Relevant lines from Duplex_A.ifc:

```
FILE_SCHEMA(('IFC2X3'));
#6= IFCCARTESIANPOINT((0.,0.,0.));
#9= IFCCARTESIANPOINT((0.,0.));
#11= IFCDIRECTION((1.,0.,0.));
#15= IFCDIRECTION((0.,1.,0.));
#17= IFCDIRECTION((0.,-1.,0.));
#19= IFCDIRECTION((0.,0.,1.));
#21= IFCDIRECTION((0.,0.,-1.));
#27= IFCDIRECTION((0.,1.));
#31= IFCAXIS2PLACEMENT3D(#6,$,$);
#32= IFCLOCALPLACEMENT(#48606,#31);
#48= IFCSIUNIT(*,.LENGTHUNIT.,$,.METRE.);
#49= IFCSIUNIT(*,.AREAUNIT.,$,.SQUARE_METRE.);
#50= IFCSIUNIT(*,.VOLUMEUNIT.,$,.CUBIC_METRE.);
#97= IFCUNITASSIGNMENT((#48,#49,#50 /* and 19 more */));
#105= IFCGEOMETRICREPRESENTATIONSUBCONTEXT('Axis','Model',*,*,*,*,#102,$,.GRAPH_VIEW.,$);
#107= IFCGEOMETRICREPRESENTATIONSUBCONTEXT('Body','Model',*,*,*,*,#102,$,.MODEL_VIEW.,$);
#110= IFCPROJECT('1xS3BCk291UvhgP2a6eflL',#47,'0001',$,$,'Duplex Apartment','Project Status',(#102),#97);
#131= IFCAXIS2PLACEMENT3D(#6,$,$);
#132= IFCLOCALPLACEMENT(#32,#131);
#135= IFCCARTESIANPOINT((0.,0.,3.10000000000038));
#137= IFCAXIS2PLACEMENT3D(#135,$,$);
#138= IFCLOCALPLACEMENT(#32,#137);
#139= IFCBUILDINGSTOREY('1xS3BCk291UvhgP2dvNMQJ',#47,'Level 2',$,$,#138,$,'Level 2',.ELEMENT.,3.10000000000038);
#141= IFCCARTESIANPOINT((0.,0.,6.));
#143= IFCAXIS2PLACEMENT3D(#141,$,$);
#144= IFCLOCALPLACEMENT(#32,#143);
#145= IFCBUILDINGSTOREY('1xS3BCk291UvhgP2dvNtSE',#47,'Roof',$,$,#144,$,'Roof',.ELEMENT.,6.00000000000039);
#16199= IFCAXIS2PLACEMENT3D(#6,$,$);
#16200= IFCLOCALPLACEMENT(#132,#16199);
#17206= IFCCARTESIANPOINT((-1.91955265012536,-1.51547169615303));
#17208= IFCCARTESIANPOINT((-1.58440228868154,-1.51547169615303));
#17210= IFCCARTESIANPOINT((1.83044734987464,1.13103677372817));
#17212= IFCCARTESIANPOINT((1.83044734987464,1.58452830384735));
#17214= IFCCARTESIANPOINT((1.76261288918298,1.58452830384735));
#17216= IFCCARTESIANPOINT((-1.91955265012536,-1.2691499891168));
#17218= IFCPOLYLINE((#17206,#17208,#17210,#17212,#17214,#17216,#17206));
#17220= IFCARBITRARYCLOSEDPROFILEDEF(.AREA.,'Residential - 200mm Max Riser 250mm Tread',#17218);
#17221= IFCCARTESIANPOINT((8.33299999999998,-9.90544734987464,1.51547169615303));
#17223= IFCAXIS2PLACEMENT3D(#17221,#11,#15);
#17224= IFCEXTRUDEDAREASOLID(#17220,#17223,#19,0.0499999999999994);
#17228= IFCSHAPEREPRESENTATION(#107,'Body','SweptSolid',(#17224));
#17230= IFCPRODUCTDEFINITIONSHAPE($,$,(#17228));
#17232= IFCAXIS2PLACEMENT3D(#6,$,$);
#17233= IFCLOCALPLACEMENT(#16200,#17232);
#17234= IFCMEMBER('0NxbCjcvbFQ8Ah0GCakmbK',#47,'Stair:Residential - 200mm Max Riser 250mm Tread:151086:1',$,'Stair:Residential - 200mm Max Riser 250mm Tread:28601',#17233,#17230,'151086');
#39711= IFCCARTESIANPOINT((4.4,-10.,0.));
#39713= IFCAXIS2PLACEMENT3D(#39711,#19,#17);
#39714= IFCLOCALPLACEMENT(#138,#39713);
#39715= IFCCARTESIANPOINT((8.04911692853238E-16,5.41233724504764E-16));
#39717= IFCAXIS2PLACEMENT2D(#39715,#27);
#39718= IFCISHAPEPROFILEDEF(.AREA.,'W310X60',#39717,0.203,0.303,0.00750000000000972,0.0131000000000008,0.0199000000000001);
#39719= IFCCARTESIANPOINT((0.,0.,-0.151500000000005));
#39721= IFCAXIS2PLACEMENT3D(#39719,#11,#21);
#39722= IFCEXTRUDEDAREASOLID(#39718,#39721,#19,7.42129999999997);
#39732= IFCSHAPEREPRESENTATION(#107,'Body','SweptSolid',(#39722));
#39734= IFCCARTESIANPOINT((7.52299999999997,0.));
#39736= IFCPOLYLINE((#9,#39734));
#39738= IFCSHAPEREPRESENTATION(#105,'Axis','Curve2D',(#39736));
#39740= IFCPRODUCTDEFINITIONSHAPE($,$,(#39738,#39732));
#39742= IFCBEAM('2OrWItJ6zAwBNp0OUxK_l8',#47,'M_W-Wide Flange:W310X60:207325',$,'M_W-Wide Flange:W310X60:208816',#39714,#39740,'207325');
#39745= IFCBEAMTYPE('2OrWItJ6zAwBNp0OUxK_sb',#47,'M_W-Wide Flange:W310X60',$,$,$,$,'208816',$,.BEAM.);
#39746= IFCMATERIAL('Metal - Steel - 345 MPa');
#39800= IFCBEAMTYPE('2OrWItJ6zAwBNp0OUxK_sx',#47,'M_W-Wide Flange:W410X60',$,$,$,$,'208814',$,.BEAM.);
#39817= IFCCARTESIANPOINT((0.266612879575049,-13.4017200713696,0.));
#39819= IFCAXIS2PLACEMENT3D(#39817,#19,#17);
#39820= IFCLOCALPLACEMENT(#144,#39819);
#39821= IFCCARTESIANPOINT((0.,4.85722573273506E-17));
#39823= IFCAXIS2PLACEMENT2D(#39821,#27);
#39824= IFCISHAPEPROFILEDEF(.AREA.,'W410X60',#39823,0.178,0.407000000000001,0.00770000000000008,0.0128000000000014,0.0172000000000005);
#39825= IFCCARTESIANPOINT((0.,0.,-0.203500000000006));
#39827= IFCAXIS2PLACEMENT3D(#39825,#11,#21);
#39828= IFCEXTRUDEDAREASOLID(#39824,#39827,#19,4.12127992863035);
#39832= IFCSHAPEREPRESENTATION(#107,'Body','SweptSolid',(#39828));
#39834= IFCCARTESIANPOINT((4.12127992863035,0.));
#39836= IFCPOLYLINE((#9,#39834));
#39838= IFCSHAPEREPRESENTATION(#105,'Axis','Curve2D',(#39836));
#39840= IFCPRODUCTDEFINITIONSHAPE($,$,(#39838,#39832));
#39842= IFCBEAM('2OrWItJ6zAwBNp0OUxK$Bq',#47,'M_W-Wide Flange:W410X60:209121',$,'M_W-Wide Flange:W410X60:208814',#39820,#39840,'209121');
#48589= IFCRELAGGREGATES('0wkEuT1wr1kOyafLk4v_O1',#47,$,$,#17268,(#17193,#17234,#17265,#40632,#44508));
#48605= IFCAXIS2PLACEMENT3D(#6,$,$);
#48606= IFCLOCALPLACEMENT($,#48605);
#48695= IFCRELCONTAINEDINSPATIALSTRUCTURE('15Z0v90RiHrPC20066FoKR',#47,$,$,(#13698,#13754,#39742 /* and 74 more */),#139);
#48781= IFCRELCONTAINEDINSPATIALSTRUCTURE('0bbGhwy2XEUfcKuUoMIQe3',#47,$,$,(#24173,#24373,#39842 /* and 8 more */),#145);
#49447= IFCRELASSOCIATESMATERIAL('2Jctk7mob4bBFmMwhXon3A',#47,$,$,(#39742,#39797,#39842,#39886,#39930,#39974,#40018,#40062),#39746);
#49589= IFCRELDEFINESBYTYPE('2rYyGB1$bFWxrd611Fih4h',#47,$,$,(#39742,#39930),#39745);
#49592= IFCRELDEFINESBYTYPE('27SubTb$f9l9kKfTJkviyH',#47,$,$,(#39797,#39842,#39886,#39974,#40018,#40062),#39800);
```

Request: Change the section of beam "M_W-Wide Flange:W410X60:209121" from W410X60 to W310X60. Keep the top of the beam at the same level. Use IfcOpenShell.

```python
import ifcopenshell
import ifcopenshell.api.type
import ifcopenshell.util.element
import ifcopenshell.util.representation

model = ifcopenshell.open("Duplex_A.ifc")

member = model.by_guid("2OrWItJ6zAwBNp0OUxK$Bq")
source = next(p for p in model.by_type("IfcIShapeProfileDef") if p.ProfileName == "W310X60")

body = ifcopenshell.util.representation.get_representation(member, "Model", "Body")
solid = body.Items[0]
old_profile = solid.SweptArea

# Copy the section's sizes but keep this member's own profile position.
profile = ifcopenshell.util.element.copy(model, source)
# Profiles are centred, so shift by half the change in depth to hold the top.
shift = (old_profile.OverallDepth - profile.OverallDepth) / 2
x, y = old_profile.Position.Location.Coordinates
up = (-1.0, 0.0)  # upwards, in the solid's own plane
location = model.createIfcCartesianPoint((x + up[0] * shift, y + up[1] * shift))
profile.Position = model.createIfcAxis2Placement2D(location, old_profile.Position.RefDirection)
solid.SweptArea = profile
if not model.get_total_inverses(old_profile):
    ifcopenshell.util.element.remove_deep2(model, old_profile)

new_type = model.by_guid("2OrWItJ6zAwBNp0OUxK_sb")
ifcopenshell.api.type.assign_type(
    model, related_objects=[member], relating_type=new_type, should_map_representations=False
)
member.Name = member.Name.replace("W410X60", "W310X60")
member.ObjectType = "M_W-Wide Flange:W310X60:208814"

print(solid.SweptArea)

model.write("Duplex_A-out.ifc")
```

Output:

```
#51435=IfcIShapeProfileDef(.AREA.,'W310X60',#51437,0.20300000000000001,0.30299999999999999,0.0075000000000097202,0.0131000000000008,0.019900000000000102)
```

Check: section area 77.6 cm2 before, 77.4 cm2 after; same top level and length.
